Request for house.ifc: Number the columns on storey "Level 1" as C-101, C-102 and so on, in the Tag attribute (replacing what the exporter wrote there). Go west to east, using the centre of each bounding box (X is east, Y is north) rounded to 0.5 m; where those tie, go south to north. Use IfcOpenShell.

First a look at what the model holds.

```python
import ifcopenshell
import ifcopenshell.util.element
import ifcopenshell.util.placement

model = ifcopenshell.open("house.ifc")
print(model.schema)
storey = next(s for s in model.by_type("IfcBuildingStorey") if s.Name == "Level 1")
columns = [e for e in ifcopenshell.util.element.get_decomposition(storey) if e.is_a("IfcColumn")]
for e in sorted(columns, key=lambda e: e.id()):
    origin = ifcopenshell.util.placement.get_local_placement(e.ObjectPlacement)[:3, 3]
    print(e.id(), e.Tag, e.Name, origin.round(2) + 0.0, sep=" | ")
```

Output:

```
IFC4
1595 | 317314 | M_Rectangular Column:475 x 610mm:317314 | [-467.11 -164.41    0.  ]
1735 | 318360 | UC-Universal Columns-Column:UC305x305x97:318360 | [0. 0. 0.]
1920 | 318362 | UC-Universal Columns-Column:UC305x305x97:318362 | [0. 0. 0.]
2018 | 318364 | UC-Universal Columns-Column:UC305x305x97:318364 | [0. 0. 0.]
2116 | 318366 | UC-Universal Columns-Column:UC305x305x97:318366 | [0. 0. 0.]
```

```python
import ifcopenshell
import ifcopenshell.geom
import ifcopenshell.util.element
import ifcopenshell.util.shape

model = ifcopenshell.open("house.ifc")
settings = ifcopenshell.geom.settings()
settings.set("use-world-coords", True)


def centre(element):
    shape = ifcopenshell.geom.create_shape(settings, element)
    return ifcopenshell.util.shape.get_bbox_centroid(shape.geometry)


storey = next(s for s in model.by_type("IfcBuildingStorey") if s.Name == "Level 1")
columns = [e for e in ifcopenshell.util.element.get_decomposition(storey) if e.is_a("IfcColumn")]

# Insertion points can sit at a corner or the storey origin, so sort by the geometry (in metres).
centres = {e: centre(e) for e in columns}
columns.sort(key=lambda e: (round(centres[e][0] / 0.5), centres[e][1]))

for i, e in enumerate(columns, start=1):
    number = f"C-1{i:02d}"
    e.Tag = number
    print(e.id(), number)

model.write("house_rev.ifc")
```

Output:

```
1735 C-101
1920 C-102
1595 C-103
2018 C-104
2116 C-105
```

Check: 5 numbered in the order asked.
